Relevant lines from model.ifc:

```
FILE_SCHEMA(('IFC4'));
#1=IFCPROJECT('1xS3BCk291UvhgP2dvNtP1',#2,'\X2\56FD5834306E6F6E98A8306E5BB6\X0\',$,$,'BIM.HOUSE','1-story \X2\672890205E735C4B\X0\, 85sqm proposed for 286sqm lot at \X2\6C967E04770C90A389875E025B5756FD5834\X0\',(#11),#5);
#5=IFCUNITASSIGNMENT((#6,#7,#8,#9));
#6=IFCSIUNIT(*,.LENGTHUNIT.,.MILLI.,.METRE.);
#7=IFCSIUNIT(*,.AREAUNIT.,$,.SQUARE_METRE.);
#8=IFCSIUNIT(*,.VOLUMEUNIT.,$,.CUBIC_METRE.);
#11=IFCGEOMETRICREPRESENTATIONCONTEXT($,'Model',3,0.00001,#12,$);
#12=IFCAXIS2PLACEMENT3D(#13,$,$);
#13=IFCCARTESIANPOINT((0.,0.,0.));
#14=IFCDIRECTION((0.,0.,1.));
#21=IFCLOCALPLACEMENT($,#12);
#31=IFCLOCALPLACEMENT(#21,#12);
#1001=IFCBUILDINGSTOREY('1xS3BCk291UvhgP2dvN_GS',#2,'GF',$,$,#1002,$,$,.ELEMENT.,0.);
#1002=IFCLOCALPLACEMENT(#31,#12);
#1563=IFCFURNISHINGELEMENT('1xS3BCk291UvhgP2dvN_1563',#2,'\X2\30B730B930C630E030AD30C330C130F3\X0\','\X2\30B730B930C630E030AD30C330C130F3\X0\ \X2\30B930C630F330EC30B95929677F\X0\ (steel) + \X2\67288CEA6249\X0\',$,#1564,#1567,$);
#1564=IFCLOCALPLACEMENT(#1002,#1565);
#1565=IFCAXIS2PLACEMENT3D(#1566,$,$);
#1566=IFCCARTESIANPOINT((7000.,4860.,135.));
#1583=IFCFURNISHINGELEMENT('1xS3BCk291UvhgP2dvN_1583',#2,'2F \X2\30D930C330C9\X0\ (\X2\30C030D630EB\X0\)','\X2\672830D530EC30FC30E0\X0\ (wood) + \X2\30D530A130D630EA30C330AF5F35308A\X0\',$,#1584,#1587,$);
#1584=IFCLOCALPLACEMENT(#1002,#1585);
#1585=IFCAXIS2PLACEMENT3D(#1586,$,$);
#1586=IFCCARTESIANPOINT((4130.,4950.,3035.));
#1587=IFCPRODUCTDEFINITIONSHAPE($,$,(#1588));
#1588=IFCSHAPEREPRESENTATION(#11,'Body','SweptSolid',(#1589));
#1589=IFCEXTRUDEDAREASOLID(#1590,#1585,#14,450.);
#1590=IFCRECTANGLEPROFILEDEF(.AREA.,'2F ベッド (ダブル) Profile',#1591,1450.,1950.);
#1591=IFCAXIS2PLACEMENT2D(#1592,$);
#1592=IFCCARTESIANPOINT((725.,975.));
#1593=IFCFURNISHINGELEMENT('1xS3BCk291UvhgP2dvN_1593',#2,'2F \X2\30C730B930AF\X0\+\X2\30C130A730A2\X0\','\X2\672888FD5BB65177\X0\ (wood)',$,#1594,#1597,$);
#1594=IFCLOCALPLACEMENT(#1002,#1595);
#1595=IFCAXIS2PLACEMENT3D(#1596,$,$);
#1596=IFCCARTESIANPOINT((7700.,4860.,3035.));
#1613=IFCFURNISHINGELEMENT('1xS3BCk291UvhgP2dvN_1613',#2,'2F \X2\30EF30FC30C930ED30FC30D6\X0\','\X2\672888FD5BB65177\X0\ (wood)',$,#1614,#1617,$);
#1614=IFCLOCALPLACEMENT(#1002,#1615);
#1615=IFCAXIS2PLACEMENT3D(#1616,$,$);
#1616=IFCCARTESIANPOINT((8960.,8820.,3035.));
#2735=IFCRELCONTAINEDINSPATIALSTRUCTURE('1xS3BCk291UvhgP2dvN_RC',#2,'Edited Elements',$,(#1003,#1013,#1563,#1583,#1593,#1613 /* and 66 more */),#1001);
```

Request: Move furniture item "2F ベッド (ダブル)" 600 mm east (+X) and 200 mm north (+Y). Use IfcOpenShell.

```python
import ifcopenshell
import ifcopenshell.api.geometry
import ifcopenshell.util.placement
import ifcopenshell.util.unit

model = ifcopenshell.open("model.ifc")
unit_scale = ifcopenshell.util.unit.calculate_unit_scale(model)

item = model.by_id(1583)
matrix = ifcopenshell.util.placement.get_local_placement(item.ObjectPlacement)
matrix[0, 3] += 0.6 / unit_scale
matrix[1, 3] += 0.2 / unit_scale
ifcopenshell.api.geometry.edit_object_placement(model, product=item, matrix=matrix, is_si=False)

print(ifcopenshell.util.placement.get_local_placement(item.ObjectPlacement).round(3) + 0.0)

model.write("model_updated.ifc")
```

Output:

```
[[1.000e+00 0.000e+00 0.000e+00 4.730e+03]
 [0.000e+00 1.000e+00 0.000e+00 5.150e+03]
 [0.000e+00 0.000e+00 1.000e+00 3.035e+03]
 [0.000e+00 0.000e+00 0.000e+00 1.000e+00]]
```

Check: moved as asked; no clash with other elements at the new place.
